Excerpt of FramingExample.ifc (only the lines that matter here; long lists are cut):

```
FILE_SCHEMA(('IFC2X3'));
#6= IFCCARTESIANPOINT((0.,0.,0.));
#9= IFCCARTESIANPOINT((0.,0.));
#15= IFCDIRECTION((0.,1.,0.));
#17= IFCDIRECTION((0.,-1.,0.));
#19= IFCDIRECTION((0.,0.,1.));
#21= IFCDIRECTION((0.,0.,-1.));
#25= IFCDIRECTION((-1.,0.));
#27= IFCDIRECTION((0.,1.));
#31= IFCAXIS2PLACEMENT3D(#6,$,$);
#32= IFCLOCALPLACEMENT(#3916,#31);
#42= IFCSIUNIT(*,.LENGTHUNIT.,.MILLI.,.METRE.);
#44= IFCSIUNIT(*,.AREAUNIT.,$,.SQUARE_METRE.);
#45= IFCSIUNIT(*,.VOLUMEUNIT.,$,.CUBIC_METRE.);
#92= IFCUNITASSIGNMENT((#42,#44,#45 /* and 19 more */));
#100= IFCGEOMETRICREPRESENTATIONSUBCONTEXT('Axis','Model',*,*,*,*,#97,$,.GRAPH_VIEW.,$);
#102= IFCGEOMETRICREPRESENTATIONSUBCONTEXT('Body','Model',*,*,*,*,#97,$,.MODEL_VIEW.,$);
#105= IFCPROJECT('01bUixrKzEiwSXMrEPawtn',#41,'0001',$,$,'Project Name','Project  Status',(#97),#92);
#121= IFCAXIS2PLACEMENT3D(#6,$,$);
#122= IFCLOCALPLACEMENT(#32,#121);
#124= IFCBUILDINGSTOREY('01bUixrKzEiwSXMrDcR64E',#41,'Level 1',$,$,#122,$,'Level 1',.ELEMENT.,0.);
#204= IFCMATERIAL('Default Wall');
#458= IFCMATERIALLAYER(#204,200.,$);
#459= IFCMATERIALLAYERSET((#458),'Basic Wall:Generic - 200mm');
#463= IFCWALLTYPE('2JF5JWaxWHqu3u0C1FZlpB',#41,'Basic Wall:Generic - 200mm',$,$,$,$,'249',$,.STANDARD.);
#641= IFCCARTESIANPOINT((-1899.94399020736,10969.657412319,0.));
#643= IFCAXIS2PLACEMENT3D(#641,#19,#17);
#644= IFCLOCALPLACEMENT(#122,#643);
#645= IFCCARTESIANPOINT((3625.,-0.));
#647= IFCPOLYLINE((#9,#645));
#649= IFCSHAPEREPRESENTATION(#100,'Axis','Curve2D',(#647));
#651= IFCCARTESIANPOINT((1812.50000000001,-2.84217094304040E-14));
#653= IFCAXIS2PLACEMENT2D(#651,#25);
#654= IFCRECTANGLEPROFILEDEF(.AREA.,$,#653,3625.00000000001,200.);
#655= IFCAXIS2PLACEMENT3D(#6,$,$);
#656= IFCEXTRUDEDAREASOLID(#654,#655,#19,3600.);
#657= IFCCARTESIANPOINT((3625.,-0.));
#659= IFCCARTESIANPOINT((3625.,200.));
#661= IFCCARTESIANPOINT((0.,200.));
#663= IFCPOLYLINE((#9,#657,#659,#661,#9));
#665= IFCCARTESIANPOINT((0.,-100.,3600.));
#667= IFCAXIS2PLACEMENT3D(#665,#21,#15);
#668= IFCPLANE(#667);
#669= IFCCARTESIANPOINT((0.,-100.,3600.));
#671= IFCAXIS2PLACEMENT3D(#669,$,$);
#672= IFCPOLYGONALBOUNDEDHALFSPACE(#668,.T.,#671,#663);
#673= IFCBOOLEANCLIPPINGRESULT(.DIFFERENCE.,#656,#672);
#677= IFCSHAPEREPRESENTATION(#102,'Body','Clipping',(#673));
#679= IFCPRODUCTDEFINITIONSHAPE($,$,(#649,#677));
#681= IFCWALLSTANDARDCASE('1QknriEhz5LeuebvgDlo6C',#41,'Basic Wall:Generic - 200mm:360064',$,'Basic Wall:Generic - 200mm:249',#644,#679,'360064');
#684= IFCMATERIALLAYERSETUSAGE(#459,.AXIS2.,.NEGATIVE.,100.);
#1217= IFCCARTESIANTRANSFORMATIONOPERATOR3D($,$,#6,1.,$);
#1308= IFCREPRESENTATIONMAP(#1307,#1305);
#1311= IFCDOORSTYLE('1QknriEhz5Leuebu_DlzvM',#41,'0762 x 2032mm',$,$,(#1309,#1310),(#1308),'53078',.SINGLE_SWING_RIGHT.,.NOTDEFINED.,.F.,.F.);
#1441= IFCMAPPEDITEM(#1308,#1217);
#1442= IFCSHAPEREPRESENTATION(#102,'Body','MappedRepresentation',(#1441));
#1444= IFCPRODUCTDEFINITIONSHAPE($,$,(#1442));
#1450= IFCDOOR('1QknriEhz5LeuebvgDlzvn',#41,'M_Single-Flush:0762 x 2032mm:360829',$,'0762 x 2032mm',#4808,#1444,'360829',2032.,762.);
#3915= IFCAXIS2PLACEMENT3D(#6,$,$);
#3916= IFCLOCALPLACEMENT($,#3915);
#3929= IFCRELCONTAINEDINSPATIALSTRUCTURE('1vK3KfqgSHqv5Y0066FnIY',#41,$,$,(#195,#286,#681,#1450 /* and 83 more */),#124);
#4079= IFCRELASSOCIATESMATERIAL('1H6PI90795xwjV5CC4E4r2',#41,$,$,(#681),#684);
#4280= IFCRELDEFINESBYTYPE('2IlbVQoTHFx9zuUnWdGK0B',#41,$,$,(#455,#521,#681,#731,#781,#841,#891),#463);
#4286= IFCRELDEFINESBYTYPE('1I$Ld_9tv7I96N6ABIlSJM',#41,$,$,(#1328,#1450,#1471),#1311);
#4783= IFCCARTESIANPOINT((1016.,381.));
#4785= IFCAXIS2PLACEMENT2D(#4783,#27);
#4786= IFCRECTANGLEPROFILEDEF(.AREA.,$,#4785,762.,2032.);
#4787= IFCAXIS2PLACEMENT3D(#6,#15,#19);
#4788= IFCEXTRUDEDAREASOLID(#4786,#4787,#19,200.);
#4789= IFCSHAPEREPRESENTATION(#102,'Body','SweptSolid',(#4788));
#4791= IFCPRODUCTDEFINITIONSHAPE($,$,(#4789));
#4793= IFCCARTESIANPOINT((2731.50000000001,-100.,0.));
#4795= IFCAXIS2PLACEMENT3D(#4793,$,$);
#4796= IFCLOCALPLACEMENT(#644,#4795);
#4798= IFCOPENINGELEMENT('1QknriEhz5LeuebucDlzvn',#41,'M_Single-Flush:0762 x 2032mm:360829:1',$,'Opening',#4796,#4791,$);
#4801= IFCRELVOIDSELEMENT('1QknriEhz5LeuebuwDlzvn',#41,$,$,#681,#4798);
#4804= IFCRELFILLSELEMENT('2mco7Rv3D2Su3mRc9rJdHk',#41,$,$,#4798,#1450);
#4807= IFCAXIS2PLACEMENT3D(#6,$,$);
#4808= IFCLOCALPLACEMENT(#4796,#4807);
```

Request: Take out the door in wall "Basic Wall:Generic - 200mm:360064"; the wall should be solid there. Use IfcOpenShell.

```python
import ifcopenshell
import ifcopenshell.api.feature
import ifcopenshell.api.root
import ifcopenshell.geom
import ifcopenshell.util.shape

model = ifcopenshell.open("FramingExample.ifc")
settings = ifcopenshell.geom.settings()


def volume(element):
    """Net volume in cubic metres, openings subtracted."""
    shape = ifcopenshell.geom.create_shape(settings, element)
    return ifcopenshell.util.shape.get_volume(shape.geometry)


door = model.by_guid("1QknriEhz5LeuebvgDlzvn")
opening = door.FillsVoids[0].RelatingOpeningElement
wall = opening.VoidsElements[0].RelatingBuildingElement
before = volume(wall)

ifcopenshell.api.root.remove_product(model, product=door)
ifcopenshell.api.feature.remove_feature(model, feature=opening)

after = volume(wall)

print(f"wall volume {before:.3f} -> {after:.3f} m3")

model.write("FramingExample_v2.ifc")
```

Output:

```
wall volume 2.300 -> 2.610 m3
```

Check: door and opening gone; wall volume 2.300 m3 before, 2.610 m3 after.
